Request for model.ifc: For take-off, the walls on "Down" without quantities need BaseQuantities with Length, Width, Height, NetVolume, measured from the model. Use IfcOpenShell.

First a look at what the model holds.

```python
import ifcopenshell
import ifcopenshell.util.element
import ifcopenshell.util.unit

model = ifcopenshell.open("model.ifc")
print(model.schema)
for unit_type in ("LENGTHUNIT", "AREAUNIT", "VOLUMEUNIT"):
    print(unit_type, ifcopenshell.util.unit.calculate_unit_scale(model, unit_type))
storey = next(s for s in model.by_type("IfcBuildingStorey") if s.Name == "Down")
walls = [e for e in ifcopenshell.util.element.get_decomposition(storey) if e.is_a("IfcWall")]
for e in sorted(walls, key=lambda e: e.id()):
    print(e.id(), e.is_a(), e.Name, list(ifcopenshell.util.element.get_psets(e, qtos_only=True)), sep=" | ")
```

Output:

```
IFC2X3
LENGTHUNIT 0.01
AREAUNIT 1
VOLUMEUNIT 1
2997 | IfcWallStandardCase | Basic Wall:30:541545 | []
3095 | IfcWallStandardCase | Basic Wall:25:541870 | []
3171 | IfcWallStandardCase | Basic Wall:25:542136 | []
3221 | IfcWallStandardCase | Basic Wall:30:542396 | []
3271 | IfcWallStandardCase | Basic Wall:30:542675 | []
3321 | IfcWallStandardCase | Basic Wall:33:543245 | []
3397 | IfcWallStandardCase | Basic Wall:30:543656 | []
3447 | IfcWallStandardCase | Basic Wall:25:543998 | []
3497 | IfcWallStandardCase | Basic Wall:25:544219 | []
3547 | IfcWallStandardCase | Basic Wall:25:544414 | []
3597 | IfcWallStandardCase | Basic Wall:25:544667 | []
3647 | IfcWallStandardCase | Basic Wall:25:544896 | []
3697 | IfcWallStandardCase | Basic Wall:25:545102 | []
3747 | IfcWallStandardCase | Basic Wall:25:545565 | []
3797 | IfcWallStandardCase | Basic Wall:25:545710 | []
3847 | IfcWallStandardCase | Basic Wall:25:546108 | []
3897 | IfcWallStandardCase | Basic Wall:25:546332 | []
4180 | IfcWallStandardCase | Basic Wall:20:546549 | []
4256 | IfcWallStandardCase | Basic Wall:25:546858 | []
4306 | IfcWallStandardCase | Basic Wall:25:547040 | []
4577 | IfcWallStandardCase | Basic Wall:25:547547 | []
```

```python
import ifcopenshell
import ifcopenshell.api.pset
import ifcopenshell.geom
import ifcopenshell.util.element
import ifcopenshell.util.shape
import ifcopenshell.util.unit

model = ifcopenshell.open("model.ifc")
unit_scale = ifcopenshell.util.unit.calculate_unit_scale(model)
volume_scale = ifcopenshell.util.unit.calculate_unit_scale(model, "VOLUMEUNIT")
settings = ifcopenshell.geom.settings()

storey = next(s for s in model.by_type("IfcBuildingStorey") if s.Name == "Down")
walls = [e for e in ifcopenshell.util.element.get_decomposition(storey) if e.is_a("IfcWall")]

for e in sorted(walls, key=lambda e: e.id()):
    if ifcopenshell.util.element.get_psets(e, qtos_only=True, should_inherit=False):
        continue
    # Geometry comes back in metres, in the element's own axes.
    shape = ifcopenshell.geom.create_shape(settings, e)
    values = {
        "Length": ifcopenshell.util.shape.get_x(shape.geometry) / unit_scale,
        "Width": ifcopenshell.util.shape.get_y(shape.geometry) / unit_scale,
        "Height": ifcopenshell.util.shape.get_z(shape.geometry) / unit_scale,
        "NetVolume": ifcopenshell.util.shape.get_volume(shape.geometry) / volume_scale,
    }
    qto = ifcopenshell.api.pset.add_qto(model, product=e, name="BaseQuantities")
    ifcopenshell.api.pset.edit_qto(model, qto=qto, properties=values)
    print(e.id(), {k: round(v, 3) for k, v in values.items()})

model.write("model_rev.ifc")
```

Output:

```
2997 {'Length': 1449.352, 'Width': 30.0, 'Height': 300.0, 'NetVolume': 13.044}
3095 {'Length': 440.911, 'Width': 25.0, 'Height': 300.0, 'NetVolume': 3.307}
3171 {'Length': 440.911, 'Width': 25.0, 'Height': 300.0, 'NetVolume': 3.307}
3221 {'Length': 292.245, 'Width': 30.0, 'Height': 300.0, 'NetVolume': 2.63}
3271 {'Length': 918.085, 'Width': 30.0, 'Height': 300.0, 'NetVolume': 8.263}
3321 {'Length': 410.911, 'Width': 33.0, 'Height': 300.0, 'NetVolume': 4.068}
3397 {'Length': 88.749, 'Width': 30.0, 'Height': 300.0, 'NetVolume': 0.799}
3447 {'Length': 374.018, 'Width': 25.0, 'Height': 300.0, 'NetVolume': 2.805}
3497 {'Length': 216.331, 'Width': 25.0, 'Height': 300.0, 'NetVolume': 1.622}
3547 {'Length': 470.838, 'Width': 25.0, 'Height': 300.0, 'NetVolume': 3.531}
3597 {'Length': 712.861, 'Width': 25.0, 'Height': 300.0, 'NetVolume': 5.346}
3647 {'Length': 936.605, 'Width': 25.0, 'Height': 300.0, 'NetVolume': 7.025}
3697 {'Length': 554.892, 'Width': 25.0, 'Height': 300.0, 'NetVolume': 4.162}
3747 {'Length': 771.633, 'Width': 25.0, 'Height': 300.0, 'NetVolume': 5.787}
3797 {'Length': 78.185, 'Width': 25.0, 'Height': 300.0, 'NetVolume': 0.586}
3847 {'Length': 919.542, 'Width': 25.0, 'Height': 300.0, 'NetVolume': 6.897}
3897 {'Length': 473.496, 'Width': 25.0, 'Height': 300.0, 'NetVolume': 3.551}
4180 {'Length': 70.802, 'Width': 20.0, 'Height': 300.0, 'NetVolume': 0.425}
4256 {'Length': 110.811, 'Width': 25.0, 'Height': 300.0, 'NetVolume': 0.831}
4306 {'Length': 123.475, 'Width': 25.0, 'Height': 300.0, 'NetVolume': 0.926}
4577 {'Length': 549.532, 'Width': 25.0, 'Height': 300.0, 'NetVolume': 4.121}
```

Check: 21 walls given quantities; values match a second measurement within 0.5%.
